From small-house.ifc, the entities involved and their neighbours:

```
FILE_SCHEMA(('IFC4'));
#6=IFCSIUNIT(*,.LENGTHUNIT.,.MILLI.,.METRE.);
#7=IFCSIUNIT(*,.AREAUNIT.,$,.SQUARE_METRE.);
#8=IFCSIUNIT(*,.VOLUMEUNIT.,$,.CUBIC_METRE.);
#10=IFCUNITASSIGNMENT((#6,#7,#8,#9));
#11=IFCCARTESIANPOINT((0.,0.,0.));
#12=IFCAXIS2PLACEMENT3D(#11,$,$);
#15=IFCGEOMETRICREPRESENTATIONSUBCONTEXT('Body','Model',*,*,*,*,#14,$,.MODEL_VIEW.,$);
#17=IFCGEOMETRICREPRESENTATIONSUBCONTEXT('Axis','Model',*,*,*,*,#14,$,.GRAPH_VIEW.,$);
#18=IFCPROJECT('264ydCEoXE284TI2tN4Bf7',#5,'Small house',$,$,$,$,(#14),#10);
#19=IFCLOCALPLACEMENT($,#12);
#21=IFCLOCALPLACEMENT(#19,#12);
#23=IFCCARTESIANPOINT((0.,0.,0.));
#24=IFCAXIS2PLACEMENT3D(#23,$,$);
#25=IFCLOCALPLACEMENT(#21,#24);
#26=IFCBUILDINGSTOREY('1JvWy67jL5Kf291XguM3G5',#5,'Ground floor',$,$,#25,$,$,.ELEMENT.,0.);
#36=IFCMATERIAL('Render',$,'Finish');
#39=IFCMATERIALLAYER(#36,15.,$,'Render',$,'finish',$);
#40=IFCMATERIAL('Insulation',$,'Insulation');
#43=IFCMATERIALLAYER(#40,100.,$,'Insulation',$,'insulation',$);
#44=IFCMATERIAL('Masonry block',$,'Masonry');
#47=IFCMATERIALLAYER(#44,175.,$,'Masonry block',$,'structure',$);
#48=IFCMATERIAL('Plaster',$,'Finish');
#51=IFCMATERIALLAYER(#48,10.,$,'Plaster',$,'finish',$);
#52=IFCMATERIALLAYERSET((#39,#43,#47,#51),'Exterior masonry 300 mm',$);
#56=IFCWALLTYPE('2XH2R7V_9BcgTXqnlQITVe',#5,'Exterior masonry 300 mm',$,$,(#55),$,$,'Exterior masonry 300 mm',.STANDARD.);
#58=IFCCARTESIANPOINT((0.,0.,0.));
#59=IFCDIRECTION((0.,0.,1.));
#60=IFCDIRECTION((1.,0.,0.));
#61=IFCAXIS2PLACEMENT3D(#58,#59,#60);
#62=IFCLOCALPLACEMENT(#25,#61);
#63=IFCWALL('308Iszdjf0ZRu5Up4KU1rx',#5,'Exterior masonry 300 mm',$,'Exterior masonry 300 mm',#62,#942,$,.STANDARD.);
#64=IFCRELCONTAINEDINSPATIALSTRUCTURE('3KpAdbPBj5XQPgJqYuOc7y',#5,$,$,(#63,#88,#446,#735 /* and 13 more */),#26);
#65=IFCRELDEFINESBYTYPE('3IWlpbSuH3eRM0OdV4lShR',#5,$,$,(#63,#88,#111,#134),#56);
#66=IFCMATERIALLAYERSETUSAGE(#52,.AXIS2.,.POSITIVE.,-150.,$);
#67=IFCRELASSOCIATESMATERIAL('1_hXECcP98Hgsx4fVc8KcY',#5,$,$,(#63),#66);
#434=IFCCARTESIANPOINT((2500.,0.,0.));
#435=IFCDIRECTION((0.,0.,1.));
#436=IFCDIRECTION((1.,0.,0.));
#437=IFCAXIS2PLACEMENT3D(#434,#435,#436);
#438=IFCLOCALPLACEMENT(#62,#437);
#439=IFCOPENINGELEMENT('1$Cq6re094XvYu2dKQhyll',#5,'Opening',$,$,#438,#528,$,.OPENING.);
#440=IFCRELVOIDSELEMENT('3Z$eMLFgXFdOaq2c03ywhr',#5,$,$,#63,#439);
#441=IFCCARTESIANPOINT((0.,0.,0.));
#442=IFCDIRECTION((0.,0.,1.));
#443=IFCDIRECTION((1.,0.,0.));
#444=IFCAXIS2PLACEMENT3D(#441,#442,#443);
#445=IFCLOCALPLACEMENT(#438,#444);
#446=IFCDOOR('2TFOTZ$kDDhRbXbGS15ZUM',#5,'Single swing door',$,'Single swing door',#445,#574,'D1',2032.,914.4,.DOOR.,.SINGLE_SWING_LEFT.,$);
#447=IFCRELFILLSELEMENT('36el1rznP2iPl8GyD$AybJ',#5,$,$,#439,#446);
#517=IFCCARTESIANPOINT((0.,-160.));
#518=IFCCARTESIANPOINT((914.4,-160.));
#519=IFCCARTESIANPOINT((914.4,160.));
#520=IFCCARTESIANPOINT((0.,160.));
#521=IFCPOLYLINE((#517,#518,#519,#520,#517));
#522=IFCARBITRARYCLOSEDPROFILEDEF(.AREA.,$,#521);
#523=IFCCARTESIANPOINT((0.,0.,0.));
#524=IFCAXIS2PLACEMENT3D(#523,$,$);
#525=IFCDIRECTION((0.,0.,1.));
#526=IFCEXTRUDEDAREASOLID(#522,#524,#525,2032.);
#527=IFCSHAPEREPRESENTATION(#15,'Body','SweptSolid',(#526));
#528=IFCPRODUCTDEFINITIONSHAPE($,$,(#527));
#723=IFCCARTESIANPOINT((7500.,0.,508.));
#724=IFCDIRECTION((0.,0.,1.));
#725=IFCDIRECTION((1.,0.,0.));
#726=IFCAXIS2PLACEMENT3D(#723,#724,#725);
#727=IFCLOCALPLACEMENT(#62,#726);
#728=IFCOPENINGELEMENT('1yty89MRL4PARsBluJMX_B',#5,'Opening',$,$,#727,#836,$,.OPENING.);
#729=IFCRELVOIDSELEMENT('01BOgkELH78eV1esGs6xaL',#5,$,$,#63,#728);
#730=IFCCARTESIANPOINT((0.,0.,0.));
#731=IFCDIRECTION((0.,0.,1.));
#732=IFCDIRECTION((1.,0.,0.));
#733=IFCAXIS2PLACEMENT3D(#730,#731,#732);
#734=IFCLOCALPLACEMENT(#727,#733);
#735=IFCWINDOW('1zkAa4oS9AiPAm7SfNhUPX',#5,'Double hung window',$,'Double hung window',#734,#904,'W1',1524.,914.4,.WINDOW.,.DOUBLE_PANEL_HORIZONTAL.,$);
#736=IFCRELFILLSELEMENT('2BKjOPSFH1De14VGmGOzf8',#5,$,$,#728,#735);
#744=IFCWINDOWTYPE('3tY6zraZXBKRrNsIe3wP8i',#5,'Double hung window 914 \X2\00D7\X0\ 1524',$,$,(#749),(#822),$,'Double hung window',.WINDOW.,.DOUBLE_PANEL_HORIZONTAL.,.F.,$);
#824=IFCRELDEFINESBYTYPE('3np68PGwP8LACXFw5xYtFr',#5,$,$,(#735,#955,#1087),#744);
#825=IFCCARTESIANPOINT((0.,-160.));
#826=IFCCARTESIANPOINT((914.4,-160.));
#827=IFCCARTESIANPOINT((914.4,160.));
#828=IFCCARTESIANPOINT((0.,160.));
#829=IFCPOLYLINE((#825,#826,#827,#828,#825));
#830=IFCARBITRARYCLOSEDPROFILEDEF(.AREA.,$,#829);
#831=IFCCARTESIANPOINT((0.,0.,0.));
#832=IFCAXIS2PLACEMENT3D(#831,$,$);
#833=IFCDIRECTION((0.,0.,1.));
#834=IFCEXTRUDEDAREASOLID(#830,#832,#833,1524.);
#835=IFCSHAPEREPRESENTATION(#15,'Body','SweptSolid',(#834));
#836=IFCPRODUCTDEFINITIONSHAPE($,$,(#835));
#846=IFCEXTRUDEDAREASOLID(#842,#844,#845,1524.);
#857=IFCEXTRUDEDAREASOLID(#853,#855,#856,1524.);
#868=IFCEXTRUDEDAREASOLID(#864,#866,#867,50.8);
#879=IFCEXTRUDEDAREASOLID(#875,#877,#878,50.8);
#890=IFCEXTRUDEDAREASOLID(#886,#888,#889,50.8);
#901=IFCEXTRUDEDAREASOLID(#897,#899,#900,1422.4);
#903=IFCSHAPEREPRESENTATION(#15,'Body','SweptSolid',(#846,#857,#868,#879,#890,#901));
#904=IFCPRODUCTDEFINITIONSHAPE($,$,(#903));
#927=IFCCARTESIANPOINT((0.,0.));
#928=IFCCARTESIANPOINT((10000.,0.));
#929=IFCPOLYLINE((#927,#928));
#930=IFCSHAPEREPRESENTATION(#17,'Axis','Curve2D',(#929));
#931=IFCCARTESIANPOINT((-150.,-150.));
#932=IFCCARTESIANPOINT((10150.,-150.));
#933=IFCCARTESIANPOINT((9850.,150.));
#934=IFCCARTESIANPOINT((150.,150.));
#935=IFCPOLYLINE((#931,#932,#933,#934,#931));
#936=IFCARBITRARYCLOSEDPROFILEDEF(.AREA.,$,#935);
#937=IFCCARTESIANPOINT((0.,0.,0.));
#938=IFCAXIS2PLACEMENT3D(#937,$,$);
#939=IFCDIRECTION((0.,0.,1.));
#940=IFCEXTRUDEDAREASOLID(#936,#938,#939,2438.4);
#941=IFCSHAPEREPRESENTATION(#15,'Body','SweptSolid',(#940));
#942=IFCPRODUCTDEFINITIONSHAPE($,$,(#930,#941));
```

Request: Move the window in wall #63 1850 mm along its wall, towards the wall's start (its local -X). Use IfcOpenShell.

```python
import ifcopenshell
import ifcopenshell.api.geometry
import ifcopenshell.util.placement
import ifcopenshell.util.unit

model = ifcopenshell.open("small-house.ifc")
unit_scale = ifcopenshell.util.unit.calculate_unit_scale(model)

window = model.by_guid("1zkAa4oS9AiPAm7SfNhUPX")
opening = window.FillsVoids[0].RelatingOpeningElement
wall = opening.VoidsElements[0].RelatingBuildingElement

wall_matrix = ifcopenshell.util.placement.get_local_placement(wall.ObjectPlacement)
shift = wall_matrix[:3, 0] * -1.85 / unit_scale
before = ifcopenshell.util.placement.get_local_placement(window.ObjectPlacement)[:3, 3].copy()

# The window is placed relative to its opening, so it follows when the opening moves.
matrix = ifcopenshell.util.placement.get_local_placement(opening.ObjectPlacement)
matrix[:3, 3] += shift
ifcopenshell.api.geometry.edit_object_placement(
    model, product=opening, matrix=matrix, is_si=False, should_transform_children=True
)

after = ifcopenshell.util.placement.get_local_placement(window.ObjectPlacement)[:3, 3]
print("window moved by", (after - before).round(3) + 0.0)

model.write("small-house_updated.ifc")
```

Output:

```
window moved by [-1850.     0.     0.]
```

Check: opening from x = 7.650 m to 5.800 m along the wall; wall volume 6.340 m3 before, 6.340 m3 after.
